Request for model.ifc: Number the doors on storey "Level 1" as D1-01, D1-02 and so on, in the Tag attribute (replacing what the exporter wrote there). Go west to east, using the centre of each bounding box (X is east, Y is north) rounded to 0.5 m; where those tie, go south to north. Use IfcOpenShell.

First a look at what the model holds.

```python
import ifcopenshell
import ifcopenshell.util.element
import ifcopenshell.util.placement

model = ifcopenshell.open("model.ifc")
print(model.schema)
storey = next(s for s in model.by_type("IfcBuildingStorey") if s.Name == "Level 1")
doors = [e for e in ifcopenshell.util.element.get_decomposition(storey) if e.is_a("IfcDoor")]
for e in sorted(doors, key=lambda e: e.id()):
    origin = ifcopenshell.util.placement.get_local_placement(e.ObjectPlacement)[:3, 3]
    print(e.id(), e.Tag, e.Name, origin.round(2) + 0.0, sep=" | ")
```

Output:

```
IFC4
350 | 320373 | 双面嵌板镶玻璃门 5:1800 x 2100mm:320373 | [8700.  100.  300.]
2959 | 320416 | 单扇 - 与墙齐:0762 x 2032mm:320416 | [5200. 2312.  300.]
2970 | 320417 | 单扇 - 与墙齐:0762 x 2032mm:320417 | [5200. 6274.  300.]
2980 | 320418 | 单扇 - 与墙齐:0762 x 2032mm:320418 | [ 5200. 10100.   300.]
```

```python
import ifcopenshell
import ifcopenshell.geom
import ifcopenshell.util.element
import ifcopenshell.util.shape

model = ifcopenshell.open("model.ifc")
settings = ifcopenshell.geom.settings()
settings.set("use-world-coords", True)


def centre(element):
    shape = ifcopenshell.geom.create_shape(settings, element)
    return ifcopenshell.util.shape.get_bbox_centroid(shape.geometry)


storey = next(s for s in model.by_type("IfcBuildingStorey") if s.Name == "Level 1")
doors = [e for e in ifcopenshell.util.element.get_decomposition(storey) if e.is_a("IfcDoor")]

# Insertion points can sit at a corner or the storey origin, so sort by the geometry (in metres).
centres = {e: centre(e) for e in doors}
doors.sort(key=lambda e: (round(centres[e][0] / 0.5), centres[e][1]))

for i, e in enumerate(doors, start=1):
    number = f"D1-{i:02d}"
    e.Tag = number
    print(e.id(), number)

model.write("model_v2.ifc")
```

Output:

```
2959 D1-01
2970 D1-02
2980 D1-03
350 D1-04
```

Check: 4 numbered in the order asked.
